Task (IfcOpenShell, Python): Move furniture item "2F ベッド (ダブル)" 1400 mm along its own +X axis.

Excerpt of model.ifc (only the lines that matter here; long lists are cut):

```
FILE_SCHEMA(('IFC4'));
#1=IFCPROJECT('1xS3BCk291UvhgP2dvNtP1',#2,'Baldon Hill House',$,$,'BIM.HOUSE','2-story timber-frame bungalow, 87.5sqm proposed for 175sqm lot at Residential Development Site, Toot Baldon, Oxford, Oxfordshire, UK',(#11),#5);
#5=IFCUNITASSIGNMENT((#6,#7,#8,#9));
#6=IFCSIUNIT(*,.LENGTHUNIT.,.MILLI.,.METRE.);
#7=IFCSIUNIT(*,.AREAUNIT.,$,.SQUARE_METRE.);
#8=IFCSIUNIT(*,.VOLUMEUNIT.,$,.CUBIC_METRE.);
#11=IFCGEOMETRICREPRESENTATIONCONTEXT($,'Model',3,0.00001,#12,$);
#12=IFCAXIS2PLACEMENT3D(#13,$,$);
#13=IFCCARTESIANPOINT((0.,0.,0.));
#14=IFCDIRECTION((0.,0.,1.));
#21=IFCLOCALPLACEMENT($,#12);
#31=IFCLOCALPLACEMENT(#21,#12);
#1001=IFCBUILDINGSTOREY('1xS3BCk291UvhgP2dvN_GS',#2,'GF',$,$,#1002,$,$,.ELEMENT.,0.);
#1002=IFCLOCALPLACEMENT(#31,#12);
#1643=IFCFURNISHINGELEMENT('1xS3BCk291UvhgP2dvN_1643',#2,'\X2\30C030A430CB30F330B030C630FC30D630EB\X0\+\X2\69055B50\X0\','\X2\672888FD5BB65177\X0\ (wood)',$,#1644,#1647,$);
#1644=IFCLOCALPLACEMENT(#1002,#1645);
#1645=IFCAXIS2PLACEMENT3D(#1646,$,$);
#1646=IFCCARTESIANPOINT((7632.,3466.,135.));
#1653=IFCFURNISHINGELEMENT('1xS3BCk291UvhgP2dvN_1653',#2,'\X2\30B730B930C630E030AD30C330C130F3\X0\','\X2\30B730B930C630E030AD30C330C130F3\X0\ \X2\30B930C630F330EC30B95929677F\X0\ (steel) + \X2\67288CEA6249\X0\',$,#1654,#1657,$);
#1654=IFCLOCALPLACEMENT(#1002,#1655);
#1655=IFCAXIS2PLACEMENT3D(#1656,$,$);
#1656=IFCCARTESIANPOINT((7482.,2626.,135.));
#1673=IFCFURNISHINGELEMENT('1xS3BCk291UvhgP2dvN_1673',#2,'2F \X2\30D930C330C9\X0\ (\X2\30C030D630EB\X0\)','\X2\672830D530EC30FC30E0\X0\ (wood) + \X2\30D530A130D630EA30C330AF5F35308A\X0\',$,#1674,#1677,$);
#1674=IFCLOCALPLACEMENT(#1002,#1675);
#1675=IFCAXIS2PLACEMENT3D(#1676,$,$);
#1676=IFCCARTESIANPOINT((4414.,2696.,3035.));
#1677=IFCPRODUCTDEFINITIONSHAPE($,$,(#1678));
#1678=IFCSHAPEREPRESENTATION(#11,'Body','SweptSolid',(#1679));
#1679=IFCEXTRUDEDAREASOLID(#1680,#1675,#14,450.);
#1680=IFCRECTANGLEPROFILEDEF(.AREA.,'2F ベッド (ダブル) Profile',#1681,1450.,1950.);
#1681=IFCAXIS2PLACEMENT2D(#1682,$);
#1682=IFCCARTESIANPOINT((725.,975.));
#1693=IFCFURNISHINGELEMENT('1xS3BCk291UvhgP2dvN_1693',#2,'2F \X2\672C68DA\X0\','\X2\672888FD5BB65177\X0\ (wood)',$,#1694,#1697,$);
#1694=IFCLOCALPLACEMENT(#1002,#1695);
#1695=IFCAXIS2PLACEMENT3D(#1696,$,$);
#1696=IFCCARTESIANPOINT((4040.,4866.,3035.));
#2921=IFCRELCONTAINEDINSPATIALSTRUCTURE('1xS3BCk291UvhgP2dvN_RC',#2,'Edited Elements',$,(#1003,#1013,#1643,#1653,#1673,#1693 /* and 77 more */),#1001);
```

```python
import ifcopenshell
import ifcopenshell.api.geometry
import ifcopenshell.util.placement

model = ifcopenshell.open("model.ifc")

item = model.by_id(1673)
matrix = ifcopenshell.util.placement.get_local_placement(item.ObjectPlacement)
matrix[:3, 3] += matrix[:3, 0] * 1400.0
ifcopenshell.api.geometry.edit_object_placement(model, product=item, matrix=matrix, is_si=False)

print(ifcopenshell.util.placement.get_local_placement(item.ObjectPlacement).round(3) + 0.0)

model.write("model_updated.ifc")
```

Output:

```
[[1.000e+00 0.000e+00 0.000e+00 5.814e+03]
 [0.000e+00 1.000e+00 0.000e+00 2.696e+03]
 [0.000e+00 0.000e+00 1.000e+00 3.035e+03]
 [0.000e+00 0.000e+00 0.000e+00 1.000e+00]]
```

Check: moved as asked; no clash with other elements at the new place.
